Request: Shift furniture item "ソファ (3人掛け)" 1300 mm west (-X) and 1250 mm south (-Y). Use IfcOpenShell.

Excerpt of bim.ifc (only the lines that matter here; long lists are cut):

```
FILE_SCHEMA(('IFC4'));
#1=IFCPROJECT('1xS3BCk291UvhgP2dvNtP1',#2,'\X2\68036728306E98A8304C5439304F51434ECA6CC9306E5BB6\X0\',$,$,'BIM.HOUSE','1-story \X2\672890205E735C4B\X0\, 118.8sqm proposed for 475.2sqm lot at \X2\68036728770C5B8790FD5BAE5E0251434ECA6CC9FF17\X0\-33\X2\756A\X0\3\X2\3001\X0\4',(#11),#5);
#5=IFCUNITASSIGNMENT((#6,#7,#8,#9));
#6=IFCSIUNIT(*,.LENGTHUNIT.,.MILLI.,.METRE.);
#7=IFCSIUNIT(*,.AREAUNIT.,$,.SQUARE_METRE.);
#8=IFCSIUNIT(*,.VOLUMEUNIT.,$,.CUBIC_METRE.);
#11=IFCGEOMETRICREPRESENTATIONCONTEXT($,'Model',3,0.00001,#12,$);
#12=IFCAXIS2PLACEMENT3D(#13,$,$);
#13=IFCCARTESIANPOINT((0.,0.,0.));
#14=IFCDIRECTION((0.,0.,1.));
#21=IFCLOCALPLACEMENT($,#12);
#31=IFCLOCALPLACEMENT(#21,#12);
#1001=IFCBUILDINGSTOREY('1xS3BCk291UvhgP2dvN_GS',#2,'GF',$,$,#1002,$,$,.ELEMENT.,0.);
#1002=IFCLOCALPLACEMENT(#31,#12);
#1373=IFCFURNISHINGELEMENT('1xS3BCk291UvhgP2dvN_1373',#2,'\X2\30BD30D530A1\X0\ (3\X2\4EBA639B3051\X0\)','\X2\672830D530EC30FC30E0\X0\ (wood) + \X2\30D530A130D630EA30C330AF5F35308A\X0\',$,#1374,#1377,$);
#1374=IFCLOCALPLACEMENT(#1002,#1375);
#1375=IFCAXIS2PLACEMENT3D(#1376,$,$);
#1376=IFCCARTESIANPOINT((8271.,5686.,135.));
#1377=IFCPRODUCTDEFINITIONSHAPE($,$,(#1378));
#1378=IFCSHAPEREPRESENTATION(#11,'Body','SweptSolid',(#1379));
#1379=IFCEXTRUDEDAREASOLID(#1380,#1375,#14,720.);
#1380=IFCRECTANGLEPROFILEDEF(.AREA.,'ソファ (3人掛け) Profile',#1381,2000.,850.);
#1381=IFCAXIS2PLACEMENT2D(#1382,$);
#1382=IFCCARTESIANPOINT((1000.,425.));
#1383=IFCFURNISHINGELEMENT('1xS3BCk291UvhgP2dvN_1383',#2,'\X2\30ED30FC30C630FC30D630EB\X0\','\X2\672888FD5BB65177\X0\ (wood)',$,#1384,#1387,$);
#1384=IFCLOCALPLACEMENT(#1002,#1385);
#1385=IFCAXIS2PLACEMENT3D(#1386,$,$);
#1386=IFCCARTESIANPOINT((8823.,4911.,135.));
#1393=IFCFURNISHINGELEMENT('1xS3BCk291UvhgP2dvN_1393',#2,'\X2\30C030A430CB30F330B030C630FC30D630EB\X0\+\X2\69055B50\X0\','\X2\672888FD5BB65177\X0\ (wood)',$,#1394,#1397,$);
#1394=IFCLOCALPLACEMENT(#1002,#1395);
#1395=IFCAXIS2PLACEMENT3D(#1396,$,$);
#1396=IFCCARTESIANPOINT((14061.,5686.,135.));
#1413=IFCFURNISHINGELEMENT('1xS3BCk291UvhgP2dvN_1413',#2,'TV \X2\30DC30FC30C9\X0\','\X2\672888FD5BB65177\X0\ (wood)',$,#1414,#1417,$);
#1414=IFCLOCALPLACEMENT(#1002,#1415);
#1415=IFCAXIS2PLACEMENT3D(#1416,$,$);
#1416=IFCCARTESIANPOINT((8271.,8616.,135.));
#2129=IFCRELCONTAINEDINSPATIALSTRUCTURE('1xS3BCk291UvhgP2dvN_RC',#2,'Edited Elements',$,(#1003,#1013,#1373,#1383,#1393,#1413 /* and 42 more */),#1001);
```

```python
import ifcopenshell
import ifcopenshell.api.geometry
import ifcopenshell.util.placement

model = ifcopenshell.open("bim.ifc")

item = model.by_id(1373)
matrix = ifcopenshell.util.placement.get_local_placement(item.ObjectPlacement)
matrix[0, 3] -= 1300.0
matrix[1, 3] -= 1250.0
ifcopenshell.api.geometry.edit_object_placement(model, product=item, matrix=matrix, is_si=False)

print(ifcopenshell.util.placement.get_local_placement(item.ObjectPlacement).round(3) + 0.0)

model.write("bim_edited.ifc")
```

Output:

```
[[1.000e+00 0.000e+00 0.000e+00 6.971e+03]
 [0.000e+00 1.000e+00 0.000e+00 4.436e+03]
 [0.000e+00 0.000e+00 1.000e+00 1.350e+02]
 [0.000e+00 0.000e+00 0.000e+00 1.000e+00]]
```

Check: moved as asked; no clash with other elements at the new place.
